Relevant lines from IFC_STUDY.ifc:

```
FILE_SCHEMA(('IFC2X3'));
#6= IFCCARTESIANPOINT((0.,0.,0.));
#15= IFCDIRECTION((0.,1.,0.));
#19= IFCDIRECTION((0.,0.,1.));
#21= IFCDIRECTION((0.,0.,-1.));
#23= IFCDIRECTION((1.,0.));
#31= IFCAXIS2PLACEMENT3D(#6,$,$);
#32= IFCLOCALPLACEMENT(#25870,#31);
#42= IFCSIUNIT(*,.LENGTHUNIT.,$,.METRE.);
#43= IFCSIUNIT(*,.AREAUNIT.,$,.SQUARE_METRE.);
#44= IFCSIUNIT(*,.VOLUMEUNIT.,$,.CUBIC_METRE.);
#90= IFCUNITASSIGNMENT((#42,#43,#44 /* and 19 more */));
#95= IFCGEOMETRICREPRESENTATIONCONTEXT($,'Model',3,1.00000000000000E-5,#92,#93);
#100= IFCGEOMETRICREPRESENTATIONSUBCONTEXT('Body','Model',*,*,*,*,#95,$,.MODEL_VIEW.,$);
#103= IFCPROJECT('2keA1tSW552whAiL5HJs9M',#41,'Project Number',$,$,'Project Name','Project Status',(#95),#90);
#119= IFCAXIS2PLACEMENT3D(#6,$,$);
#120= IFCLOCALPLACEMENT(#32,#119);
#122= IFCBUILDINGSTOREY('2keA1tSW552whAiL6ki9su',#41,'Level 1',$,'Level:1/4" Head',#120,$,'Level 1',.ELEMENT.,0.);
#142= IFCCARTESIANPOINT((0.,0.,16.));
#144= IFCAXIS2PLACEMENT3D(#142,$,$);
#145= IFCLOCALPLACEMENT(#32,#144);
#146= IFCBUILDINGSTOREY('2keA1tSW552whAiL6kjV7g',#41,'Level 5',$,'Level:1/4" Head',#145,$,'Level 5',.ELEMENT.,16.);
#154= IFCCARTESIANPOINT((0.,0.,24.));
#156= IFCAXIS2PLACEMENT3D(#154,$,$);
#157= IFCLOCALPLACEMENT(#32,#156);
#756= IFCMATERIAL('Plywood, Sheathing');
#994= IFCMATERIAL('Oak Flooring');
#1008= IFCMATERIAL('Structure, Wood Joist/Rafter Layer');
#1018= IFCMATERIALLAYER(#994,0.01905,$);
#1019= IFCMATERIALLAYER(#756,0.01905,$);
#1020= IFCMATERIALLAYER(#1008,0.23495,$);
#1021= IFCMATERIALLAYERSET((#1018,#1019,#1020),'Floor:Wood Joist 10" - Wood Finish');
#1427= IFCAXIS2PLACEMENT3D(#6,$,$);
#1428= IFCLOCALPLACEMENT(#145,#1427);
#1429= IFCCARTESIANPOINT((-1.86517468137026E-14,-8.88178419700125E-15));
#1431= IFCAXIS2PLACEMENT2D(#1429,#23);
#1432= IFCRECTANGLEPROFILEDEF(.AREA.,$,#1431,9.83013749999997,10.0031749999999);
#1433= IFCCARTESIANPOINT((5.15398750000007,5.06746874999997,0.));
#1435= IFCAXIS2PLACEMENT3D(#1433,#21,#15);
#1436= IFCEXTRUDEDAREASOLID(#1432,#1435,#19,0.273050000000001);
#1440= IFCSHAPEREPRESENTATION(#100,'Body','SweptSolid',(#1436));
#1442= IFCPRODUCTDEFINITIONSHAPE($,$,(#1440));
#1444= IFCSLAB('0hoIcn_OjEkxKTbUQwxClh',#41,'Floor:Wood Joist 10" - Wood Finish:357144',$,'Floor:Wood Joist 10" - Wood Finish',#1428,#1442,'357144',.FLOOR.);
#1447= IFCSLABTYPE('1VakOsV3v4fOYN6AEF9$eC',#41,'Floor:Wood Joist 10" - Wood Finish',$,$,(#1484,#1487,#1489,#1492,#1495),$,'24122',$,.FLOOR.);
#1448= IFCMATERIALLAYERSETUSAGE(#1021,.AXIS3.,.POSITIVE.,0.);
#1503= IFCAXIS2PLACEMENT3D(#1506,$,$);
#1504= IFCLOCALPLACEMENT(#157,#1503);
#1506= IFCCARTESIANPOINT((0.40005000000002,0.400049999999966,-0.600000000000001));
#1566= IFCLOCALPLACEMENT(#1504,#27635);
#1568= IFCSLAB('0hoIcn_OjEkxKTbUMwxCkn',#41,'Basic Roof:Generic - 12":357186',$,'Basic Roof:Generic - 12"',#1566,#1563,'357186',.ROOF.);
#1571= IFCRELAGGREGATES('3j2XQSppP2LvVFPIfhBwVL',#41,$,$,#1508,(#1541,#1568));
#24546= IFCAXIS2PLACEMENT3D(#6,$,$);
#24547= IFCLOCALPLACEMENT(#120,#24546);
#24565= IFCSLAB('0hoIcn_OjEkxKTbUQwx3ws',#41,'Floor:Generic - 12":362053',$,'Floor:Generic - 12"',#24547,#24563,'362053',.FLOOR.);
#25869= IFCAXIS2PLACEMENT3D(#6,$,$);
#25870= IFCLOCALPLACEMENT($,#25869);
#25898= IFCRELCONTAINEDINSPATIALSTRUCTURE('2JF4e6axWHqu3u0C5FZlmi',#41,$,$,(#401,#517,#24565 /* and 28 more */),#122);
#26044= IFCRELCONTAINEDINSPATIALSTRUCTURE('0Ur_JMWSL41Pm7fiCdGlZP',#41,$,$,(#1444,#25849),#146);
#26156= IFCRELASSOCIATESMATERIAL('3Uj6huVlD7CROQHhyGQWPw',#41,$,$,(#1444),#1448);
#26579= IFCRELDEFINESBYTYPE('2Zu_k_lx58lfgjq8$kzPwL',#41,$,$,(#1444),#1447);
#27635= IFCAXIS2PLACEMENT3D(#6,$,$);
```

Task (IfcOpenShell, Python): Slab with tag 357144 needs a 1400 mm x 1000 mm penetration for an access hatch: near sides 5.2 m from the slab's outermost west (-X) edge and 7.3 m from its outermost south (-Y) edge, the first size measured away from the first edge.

```python
import numpy as np
import ifcopenshell
import ifcopenshell.api.feature
import ifcopenshell.api.geometry
import ifcopenshell.api.root
import ifcopenshell.geom
import ifcopenshell.util.placement
import ifcopenshell.util.representation
import ifcopenshell.util.shape
import ifcopenshell.util.unit

model = ifcopenshell.open("IFC_STUDY.ifc")
unit_scale = ifcopenshell.util.unit.calculate_unit_scale(model)
settings = ifcopenshell.geom.settings()


def volume(element):
    """Net volume in cubic metres, openings subtracted."""
    shape = ifcopenshell.geom.create_shape(settings, element)
    return ifcopenshell.util.shape.get_volume(shape.geometry)


slab = model.by_id(1444)
before = volume(slab)

# Extent in the slab's own axes, in metres. The edges named are its -X and -Y sides.
slab_shape = ifcopenshell.geom.create_shape(settings, slab)
vertices = ifcopenshell.util.shape.get_vertices(slab_shape.geometry)
x_min, y_min, bottom = vertices.min(axis=0)
top = vertices[:, 2].max()

opening = ifcopenshell.api.root.create_entity(model, ifc_class="IfcOpeningElement", name="Access hatch opening")
context = ifcopenshell.util.representation.get_context(model, "Model", "Body", "MODEL_VIEW")
width, depth = 1.4, 1
outline = [(0.0, 0.0), (width, 0.0), (width, depth), (0.0, depth), (0.0, 0.0)]
# Overshoot both faces by 50 mm so the cut is clean.
shape = ifcopenshell.api.geometry.add_slab_representation(
    model, context=context, depth=top - bottom + 0.1, polyline=outline
)
ifcopenshell.api.geometry.assign_representation(model, product=opening, representation=shape)

matrix = ifcopenshell.util.placement.get_local_placement(slab.ObjectPlacement)
matrix[:, 3] = matrix @ np.append(np.array([x_min + 5.2, y_min + 7.3, bottom - 0.05]) / unit_scale, 1.0)
ifcopenshell.api.geometry.edit_object_placement(model, product=opening, matrix=matrix, is_si=False)
ifcopenshell.api.feature.add_feature(model, feature=opening, element=slab)

after = volume(slab)

print(f"slab volume {before:.3f} -> {after:.3f} m3")

model.write("IFC_STUDY_v2.ifc")
```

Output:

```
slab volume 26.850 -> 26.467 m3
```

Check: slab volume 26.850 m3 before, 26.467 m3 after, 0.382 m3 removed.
